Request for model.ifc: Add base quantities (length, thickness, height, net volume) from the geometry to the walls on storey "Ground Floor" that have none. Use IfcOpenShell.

First a look at what the model holds.

```python
import ifcopenshell
import ifcopenshell.util.element
import ifcopenshell.util.unit

model = ifcopenshell.open("model.ifc")
print(model.schema)
for unit_type in ("LENGTHUNIT", "AREAUNIT", "VOLUMEUNIT"):
    print(unit_type, ifcopenshell.util.unit.calculate_unit_scale(model, unit_type))
storey = next(s for s in model.by_type("IfcBuildingStorey") if s.Name == "Ground Floor")
walls = [e for e in ifcopenshell.util.element.get_decomposition(storey) if e.is_a("IfcWall")]
for e in sorted(walls, key=lambda e: e.id()):
    print(e.id(), e.is_a(), e.Name, list(ifcopenshell.util.element.get_psets(e, qtos_only=True)), sep=" | ")
```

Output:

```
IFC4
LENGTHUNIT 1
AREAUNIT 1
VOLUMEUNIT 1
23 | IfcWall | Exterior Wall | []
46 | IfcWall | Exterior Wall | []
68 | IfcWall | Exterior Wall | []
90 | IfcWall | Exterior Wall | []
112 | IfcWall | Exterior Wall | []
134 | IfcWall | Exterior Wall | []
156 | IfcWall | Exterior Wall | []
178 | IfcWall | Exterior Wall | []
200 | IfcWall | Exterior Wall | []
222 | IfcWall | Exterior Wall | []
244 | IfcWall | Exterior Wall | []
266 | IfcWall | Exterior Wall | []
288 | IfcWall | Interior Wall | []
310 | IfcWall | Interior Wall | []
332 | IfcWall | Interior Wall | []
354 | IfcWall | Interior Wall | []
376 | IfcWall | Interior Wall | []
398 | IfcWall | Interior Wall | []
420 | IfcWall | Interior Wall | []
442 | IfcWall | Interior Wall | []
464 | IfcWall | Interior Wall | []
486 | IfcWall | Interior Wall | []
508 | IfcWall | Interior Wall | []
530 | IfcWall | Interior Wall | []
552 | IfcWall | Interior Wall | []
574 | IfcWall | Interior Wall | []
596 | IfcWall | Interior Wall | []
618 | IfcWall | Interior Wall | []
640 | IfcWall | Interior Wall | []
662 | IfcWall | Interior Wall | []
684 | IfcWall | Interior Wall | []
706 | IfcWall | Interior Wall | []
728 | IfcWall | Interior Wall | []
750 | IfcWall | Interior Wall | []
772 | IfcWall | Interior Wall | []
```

```python
import ifcopenshell
import ifcopenshell.api.pset
import ifcopenshell.geom
import ifcopenshell.util.element
import ifcopenshell.util.shape
import ifcopenshell.util.unit

model = ifcopenshell.open("model.ifc")
unit_scale = ifcopenshell.util.unit.calculate_unit_scale(model)
volume_scale = ifcopenshell.util.unit.calculate_unit_scale(model, "VOLUMEUNIT")
settings = ifcopenshell.geom.settings()

storey = next(s for s in model.by_type("IfcBuildingStorey") if s.Name == "Ground Floor")
walls = [e for e in ifcopenshell.util.element.get_decomposition(storey) if e.is_a("IfcWall")]

for e in sorted(walls, key=lambda e: e.id()):
    if ifcopenshell.util.element.get_psets(e, qtos_only=True, should_inherit=False):
        continue
    # Geometry comes back in metres, in the element's own axes.
    shape = ifcopenshell.geom.create_shape(settings, e)
    values = {
        "Length": ifcopenshell.util.shape.get_x(shape.geometry) / unit_scale,
        "Width": ifcopenshell.util.shape.get_y(shape.geometry) / unit_scale,
        "Height": ifcopenshell.util.shape.get_z(shape.geometry) / unit_scale,
        "NetVolume": ifcopenshell.util.shape.get_volume(shape.geometry) / volume_scale,
    }
    qto = ifcopenshell.api.pset.add_qto(model, product=e, name="Qto_WallBaseQuantities")
    ifcopenshell.api.pset.edit_qto(model, qto=qto, properties=values)
    print(e.id(), {k: round(v, 3) for k, v in values.items()})

model.write("model_edited.ifc")
```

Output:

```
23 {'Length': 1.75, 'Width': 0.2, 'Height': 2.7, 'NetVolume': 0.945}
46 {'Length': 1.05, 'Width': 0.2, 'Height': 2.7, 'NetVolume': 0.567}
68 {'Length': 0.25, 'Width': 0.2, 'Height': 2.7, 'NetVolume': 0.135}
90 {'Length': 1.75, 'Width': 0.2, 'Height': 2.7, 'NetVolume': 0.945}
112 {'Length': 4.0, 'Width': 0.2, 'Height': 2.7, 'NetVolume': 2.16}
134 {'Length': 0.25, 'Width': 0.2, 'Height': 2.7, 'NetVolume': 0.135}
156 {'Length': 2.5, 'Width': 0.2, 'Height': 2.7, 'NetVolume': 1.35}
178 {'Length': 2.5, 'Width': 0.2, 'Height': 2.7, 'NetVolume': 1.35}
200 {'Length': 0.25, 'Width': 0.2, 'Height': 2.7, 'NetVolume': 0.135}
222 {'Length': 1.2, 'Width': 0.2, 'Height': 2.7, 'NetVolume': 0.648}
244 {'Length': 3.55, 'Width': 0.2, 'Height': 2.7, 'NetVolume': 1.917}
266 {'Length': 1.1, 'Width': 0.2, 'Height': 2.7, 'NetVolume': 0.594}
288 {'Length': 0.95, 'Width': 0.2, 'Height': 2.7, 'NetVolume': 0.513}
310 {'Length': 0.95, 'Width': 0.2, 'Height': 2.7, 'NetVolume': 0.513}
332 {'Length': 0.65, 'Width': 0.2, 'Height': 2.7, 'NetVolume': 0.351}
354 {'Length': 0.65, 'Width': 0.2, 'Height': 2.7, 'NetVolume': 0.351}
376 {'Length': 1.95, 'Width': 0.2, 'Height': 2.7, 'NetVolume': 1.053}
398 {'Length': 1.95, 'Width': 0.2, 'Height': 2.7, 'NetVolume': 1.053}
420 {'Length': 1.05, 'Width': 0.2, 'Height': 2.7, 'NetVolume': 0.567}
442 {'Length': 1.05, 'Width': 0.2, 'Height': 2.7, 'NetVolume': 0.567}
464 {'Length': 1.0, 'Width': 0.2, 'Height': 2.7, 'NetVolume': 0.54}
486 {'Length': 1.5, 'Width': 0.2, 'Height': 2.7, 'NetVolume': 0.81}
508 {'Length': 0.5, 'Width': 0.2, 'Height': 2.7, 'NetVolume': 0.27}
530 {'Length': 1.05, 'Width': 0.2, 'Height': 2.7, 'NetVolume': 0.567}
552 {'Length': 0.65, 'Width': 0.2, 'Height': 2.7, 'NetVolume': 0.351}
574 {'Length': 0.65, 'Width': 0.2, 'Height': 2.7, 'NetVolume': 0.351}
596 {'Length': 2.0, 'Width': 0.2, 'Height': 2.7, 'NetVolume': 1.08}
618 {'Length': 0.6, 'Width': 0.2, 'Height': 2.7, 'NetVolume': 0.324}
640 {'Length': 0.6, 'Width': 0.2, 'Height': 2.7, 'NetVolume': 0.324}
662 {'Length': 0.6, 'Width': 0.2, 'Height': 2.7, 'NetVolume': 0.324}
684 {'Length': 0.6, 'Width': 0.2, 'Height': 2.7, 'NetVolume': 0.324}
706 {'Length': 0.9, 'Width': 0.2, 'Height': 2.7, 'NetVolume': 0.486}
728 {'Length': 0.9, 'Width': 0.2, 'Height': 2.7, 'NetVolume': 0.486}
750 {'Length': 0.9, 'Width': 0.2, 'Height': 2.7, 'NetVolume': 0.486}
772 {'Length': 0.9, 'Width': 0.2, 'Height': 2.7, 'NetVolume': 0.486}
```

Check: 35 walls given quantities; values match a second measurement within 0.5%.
